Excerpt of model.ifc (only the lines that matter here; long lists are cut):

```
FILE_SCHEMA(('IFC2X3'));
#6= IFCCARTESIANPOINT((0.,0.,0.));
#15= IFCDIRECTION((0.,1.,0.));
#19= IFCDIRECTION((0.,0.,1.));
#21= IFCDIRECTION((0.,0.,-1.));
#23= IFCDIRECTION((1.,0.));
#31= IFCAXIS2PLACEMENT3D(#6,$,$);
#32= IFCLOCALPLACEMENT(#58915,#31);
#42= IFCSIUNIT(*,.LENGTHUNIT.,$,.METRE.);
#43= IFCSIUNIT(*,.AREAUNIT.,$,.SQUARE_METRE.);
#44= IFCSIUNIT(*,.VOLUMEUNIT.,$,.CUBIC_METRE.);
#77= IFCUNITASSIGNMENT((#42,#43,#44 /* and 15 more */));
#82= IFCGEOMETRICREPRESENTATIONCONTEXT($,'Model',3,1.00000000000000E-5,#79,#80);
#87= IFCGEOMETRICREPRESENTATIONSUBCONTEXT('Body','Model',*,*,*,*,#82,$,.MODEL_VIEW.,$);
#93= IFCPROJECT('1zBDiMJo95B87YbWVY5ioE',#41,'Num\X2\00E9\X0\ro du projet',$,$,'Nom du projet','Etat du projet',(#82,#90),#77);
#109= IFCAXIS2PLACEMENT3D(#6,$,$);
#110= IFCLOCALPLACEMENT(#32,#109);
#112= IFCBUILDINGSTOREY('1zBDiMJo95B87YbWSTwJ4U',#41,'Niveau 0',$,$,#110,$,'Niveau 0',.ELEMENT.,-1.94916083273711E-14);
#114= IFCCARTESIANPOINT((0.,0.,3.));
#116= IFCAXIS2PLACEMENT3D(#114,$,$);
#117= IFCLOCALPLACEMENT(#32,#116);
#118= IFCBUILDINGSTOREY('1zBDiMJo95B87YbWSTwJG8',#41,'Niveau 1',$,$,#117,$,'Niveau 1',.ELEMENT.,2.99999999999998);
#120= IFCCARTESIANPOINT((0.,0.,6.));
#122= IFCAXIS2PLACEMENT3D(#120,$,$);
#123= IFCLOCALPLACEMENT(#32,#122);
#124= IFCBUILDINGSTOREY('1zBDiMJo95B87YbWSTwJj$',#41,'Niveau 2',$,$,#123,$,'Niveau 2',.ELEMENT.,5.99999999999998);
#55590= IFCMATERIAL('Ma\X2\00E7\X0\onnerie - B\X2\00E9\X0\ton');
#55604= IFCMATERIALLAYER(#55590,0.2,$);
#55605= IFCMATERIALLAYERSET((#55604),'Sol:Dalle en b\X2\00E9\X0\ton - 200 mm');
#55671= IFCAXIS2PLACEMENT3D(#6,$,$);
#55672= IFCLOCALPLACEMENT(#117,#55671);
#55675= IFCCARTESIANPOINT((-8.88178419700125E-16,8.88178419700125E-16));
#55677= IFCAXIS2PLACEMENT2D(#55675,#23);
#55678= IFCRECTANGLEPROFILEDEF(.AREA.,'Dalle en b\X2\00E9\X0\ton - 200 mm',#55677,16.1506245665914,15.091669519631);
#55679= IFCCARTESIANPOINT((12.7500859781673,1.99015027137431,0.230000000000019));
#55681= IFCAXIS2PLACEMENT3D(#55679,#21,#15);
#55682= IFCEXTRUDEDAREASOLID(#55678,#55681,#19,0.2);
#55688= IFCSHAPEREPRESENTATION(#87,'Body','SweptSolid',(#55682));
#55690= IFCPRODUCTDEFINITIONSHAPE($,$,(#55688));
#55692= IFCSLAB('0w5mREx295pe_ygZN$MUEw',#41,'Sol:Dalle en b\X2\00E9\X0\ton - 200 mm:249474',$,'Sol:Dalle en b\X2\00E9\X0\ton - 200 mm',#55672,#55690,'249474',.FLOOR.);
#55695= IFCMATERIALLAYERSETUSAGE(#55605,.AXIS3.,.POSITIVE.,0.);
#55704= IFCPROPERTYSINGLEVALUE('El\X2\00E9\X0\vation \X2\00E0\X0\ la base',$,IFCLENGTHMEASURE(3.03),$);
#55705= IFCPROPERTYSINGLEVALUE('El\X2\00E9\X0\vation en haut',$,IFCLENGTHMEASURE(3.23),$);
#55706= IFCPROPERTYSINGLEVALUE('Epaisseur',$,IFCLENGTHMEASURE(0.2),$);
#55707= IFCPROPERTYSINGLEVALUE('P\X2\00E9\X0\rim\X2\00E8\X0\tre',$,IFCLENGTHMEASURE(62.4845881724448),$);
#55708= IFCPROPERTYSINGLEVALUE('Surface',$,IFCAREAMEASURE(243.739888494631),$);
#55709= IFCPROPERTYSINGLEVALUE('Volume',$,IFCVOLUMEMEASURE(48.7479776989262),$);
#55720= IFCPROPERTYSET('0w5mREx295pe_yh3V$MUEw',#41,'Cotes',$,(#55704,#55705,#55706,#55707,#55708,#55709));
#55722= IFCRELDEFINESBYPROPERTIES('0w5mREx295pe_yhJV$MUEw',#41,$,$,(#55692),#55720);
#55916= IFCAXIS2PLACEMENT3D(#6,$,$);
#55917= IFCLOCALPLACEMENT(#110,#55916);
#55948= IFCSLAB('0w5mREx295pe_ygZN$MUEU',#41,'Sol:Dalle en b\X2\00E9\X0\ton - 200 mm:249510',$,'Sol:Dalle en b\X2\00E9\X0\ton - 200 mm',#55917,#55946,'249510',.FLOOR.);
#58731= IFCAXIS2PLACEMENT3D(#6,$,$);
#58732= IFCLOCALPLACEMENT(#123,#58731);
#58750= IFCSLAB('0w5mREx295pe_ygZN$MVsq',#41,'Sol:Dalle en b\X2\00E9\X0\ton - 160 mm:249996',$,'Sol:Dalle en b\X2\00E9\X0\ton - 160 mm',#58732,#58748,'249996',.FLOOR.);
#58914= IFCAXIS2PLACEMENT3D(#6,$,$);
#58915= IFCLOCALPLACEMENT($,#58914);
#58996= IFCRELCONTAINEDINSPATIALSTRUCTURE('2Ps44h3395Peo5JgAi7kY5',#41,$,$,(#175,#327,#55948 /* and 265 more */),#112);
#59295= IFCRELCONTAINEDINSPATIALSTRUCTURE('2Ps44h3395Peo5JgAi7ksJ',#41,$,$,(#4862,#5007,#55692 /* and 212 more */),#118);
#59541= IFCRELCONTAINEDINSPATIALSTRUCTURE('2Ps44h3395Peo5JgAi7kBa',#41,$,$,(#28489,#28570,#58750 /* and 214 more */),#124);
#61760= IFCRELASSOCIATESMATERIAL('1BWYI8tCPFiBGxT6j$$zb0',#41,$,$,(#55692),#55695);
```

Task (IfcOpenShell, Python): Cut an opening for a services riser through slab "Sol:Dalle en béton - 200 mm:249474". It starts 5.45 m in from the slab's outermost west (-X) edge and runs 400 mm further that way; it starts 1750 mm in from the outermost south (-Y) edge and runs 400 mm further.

```python
import numpy as np
import ifcopenshell
import ifcopenshell.api.feature
import ifcopenshell.api.geometry
import ifcopenshell.api.pset
import ifcopenshell.api.root
import ifcopenshell.geom
import ifcopenshell.util.element
import ifcopenshell.util.placement
import ifcopenshell.util.representation
import ifcopenshell.util.shape
import ifcopenshell.util.unit

model = ifcopenshell.open("model.ifc")
unit_scale = ifcopenshell.util.unit.calculate_unit_scale(model)
area_scale = ifcopenshell.util.unit.calculate_unit_scale(model, "AREAUNIT")
volume_scale = ifcopenshell.util.unit.calculate_unit_scale(model, "VOLUMEUNIT")
settings = ifcopenshell.geom.settings()


def volume(element):
    """Net volume in cubic metres, openings subtracted."""
    shape = ifcopenshell.geom.create_shape(settings, element)
    return ifcopenshell.util.shape.get_volume(shape.geometry)


slab = model.by_guid("0w5mREx295pe_ygZN$MUEw")
before = volume(slab)

# Extent in the slab's own axes, in metres. The edges named are its -X and -Y sides.
slab_shape = ifcopenshell.geom.create_shape(settings, slab)
vertices = ifcopenshell.util.shape.get_vertices(slab_shape.geometry)
x_min, y_min, bottom = vertices.min(axis=0)
top = vertices[:, 2].max()

opening = ifcopenshell.api.root.create_entity(model, ifc_class="IfcOpeningElement", name="Services riser opening")
context = ifcopenshell.util.representation.get_context(model, "Model", "Body", "MODEL_VIEW")
width, depth = 0.4, 0.4
outline = [(0.0, 0.0), (width, 0.0), (width, depth), (0.0, depth), (0.0, 0.0)]
# Overshoot both faces by 50 mm so the cut is clean.
shape = ifcopenshell.api.geometry.add_slab_representation(
    model, context=context, depth=top - bottom + 0.1, polyline=outline
)
ifcopenshell.api.geometry.assign_representation(model, product=opening, representation=shape)

matrix = ifcopenshell.util.placement.get_local_placement(slab.ObjectPlacement)
matrix[:, 3] = matrix @ np.append(np.array([x_min + 5.45, y_min + 1.75, bottom - 0.05]) / unit_scale, 1.0)
ifcopenshell.api.geometry.edit_object_placement(model, product=opening, matrix=matrix, is_si=False)
ifcopenshell.api.feature.add_feature(model, feature=opening, element=slab)

after = volume(slab)

# Update the slab's stored quantities.
pset = model.by_id(ifcopenshell.util.element.get_pset(slab, "Cotes", should_inherit=False)["id"])
ifcopenshell.api.pset.edit_pset(model, pset=pset, properties={
    "Surface": model.create_entity("IfcAreaMeasure", after / (top - bottom) / area_scale),
    "Volume": model.create_entity("IfcVolumeMeasure", after / volume_scale),
})

print(f"slab volume {before:.3f} -> {after:.3f} m3")

model.write("model_rev.ifc")
```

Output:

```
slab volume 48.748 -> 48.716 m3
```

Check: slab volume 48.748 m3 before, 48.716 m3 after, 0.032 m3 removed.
